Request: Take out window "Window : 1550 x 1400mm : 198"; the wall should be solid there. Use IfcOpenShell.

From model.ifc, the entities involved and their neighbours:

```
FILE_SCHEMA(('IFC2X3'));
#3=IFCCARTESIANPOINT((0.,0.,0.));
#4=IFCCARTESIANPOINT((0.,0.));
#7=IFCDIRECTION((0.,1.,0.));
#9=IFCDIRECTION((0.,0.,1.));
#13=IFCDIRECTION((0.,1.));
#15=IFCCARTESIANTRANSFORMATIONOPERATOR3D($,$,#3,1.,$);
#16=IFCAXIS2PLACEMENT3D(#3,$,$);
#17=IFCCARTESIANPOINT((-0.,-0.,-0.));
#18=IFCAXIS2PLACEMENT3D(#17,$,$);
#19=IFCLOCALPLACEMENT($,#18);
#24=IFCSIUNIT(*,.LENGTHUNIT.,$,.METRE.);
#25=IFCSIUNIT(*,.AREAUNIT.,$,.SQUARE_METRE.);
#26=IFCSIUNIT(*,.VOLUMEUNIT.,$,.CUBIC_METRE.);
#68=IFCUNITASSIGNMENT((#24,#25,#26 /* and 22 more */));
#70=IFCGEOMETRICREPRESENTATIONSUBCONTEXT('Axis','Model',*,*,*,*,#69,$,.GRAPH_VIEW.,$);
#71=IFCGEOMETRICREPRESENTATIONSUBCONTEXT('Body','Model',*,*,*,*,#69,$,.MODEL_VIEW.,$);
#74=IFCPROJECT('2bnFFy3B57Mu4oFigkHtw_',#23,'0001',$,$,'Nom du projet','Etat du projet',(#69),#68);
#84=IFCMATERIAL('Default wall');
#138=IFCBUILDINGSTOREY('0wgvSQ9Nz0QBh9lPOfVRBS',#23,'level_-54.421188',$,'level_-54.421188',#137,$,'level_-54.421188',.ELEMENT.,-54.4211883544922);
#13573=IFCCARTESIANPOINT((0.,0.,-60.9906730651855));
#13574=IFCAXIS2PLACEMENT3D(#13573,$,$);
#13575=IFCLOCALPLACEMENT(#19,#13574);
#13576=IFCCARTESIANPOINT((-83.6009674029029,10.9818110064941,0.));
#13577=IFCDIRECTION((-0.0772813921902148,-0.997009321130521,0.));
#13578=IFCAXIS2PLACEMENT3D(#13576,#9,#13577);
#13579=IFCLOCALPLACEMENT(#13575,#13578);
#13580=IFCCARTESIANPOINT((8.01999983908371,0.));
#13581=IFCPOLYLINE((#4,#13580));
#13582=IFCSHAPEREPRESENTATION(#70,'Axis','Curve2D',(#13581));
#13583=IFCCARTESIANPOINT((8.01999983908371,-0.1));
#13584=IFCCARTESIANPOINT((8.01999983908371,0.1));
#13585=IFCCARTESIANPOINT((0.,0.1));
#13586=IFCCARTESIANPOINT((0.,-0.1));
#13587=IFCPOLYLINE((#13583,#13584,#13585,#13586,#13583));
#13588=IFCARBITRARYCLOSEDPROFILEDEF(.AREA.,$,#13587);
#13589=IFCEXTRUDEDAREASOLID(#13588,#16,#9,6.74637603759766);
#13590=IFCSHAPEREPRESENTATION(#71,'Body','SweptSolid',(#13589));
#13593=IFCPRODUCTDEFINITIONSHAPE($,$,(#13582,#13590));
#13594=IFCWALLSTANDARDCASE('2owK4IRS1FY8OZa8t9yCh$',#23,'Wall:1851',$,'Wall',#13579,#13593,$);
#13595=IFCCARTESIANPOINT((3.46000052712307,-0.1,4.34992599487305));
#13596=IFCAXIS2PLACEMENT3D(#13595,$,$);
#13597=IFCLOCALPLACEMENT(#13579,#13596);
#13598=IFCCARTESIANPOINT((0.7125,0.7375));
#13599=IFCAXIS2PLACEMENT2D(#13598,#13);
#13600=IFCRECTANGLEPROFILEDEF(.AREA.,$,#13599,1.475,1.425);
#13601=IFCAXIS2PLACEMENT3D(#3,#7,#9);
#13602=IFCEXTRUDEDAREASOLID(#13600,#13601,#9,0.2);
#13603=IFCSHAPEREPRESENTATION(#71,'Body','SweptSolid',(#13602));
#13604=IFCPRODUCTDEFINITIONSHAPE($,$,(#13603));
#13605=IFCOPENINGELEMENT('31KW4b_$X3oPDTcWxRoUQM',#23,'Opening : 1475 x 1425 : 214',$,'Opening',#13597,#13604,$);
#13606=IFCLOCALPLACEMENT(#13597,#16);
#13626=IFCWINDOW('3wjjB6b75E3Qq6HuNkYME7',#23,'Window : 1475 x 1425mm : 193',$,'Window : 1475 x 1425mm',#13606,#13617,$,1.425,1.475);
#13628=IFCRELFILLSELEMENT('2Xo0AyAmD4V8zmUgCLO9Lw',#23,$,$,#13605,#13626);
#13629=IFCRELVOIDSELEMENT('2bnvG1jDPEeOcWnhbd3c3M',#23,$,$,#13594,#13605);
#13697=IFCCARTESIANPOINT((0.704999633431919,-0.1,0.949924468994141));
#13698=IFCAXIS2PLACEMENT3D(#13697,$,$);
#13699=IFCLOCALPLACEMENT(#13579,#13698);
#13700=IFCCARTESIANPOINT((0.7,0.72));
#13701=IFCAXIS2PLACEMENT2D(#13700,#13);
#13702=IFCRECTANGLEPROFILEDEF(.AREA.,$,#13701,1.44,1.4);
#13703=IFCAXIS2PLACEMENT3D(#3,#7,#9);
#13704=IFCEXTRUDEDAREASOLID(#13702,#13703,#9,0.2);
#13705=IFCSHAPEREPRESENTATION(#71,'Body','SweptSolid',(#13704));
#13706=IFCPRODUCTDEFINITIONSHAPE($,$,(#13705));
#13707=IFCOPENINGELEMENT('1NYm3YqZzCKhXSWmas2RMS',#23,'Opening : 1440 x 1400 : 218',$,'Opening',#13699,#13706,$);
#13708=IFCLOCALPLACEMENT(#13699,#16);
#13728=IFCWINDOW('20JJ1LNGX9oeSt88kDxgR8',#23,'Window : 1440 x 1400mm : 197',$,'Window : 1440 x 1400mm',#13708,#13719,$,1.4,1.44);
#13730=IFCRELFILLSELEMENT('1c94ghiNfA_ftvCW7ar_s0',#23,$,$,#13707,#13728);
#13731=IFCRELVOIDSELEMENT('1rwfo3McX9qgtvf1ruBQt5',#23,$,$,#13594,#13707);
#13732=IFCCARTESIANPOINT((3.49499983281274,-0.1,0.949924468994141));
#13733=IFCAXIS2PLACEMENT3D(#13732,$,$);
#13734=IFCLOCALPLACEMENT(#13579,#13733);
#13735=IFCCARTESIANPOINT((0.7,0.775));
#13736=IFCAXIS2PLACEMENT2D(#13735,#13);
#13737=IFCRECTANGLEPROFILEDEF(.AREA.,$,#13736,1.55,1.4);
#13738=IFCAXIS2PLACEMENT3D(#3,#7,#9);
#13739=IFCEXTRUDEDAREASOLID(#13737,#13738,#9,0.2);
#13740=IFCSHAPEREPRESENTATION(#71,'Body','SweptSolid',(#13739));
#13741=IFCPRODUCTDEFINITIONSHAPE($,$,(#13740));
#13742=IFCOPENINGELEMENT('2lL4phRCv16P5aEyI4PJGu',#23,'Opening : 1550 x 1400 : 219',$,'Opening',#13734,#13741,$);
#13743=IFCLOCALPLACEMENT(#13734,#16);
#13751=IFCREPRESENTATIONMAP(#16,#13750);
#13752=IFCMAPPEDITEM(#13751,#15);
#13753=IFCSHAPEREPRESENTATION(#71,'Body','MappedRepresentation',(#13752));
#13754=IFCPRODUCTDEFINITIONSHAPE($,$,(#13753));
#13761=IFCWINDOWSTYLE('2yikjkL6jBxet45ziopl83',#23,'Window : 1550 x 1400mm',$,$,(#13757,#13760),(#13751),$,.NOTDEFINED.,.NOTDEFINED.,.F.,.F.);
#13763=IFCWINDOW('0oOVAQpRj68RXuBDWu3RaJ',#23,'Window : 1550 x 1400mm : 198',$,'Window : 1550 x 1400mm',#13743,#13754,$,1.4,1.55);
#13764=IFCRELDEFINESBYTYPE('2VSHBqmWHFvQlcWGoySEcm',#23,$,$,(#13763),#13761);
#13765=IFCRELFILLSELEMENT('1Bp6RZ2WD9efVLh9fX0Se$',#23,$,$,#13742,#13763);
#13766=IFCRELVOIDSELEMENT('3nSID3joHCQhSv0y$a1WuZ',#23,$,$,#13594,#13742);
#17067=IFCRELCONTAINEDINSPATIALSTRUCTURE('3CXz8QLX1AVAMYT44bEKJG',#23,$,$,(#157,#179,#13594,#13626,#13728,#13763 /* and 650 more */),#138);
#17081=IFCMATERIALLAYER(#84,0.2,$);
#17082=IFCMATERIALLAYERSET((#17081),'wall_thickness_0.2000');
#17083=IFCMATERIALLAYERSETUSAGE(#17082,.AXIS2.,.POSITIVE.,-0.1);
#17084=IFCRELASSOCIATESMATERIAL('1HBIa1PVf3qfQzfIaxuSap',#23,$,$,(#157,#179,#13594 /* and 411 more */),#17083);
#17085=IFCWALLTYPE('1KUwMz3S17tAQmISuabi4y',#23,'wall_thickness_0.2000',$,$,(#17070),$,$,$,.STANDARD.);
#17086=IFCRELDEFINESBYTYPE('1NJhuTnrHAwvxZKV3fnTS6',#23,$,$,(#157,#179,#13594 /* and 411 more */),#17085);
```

```python
import ifcopenshell
import ifcopenshell.api.feature
import ifcopenshell.api.root
import ifcopenshell.geom
import ifcopenshell.util.shape

model = ifcopenshell.open("model.ifc")
settings = ifcopenshell.geom.settings()


def volume(element):
    """Net volume in cubic metres, openings subtracted."""
    shape = ifcopenshell.geom.create_shape(settings, element)
    return ifcopenshell.util.shape.get_volume(shape.geometry)


window = model.by_guid("0oOVAQpRj68RXuBDWu3RaJ")
opening = window.FillsVoids[0].RelatingOpeningElement
wall = opening.VoidsElements[0].RelatingBuildingElement
before = volume(wall)

ifcopenshell.api.root.remove_product(model, product=window)
ifcopenshell.api.feature.remove_feature(model, feature=opening)

after = volume(wall)

print(f"wall volume {before:.3f} -> {after:.3f} m3")

model.write("model_rev.ifc")
```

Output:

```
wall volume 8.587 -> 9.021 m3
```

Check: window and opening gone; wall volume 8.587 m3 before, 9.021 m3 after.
